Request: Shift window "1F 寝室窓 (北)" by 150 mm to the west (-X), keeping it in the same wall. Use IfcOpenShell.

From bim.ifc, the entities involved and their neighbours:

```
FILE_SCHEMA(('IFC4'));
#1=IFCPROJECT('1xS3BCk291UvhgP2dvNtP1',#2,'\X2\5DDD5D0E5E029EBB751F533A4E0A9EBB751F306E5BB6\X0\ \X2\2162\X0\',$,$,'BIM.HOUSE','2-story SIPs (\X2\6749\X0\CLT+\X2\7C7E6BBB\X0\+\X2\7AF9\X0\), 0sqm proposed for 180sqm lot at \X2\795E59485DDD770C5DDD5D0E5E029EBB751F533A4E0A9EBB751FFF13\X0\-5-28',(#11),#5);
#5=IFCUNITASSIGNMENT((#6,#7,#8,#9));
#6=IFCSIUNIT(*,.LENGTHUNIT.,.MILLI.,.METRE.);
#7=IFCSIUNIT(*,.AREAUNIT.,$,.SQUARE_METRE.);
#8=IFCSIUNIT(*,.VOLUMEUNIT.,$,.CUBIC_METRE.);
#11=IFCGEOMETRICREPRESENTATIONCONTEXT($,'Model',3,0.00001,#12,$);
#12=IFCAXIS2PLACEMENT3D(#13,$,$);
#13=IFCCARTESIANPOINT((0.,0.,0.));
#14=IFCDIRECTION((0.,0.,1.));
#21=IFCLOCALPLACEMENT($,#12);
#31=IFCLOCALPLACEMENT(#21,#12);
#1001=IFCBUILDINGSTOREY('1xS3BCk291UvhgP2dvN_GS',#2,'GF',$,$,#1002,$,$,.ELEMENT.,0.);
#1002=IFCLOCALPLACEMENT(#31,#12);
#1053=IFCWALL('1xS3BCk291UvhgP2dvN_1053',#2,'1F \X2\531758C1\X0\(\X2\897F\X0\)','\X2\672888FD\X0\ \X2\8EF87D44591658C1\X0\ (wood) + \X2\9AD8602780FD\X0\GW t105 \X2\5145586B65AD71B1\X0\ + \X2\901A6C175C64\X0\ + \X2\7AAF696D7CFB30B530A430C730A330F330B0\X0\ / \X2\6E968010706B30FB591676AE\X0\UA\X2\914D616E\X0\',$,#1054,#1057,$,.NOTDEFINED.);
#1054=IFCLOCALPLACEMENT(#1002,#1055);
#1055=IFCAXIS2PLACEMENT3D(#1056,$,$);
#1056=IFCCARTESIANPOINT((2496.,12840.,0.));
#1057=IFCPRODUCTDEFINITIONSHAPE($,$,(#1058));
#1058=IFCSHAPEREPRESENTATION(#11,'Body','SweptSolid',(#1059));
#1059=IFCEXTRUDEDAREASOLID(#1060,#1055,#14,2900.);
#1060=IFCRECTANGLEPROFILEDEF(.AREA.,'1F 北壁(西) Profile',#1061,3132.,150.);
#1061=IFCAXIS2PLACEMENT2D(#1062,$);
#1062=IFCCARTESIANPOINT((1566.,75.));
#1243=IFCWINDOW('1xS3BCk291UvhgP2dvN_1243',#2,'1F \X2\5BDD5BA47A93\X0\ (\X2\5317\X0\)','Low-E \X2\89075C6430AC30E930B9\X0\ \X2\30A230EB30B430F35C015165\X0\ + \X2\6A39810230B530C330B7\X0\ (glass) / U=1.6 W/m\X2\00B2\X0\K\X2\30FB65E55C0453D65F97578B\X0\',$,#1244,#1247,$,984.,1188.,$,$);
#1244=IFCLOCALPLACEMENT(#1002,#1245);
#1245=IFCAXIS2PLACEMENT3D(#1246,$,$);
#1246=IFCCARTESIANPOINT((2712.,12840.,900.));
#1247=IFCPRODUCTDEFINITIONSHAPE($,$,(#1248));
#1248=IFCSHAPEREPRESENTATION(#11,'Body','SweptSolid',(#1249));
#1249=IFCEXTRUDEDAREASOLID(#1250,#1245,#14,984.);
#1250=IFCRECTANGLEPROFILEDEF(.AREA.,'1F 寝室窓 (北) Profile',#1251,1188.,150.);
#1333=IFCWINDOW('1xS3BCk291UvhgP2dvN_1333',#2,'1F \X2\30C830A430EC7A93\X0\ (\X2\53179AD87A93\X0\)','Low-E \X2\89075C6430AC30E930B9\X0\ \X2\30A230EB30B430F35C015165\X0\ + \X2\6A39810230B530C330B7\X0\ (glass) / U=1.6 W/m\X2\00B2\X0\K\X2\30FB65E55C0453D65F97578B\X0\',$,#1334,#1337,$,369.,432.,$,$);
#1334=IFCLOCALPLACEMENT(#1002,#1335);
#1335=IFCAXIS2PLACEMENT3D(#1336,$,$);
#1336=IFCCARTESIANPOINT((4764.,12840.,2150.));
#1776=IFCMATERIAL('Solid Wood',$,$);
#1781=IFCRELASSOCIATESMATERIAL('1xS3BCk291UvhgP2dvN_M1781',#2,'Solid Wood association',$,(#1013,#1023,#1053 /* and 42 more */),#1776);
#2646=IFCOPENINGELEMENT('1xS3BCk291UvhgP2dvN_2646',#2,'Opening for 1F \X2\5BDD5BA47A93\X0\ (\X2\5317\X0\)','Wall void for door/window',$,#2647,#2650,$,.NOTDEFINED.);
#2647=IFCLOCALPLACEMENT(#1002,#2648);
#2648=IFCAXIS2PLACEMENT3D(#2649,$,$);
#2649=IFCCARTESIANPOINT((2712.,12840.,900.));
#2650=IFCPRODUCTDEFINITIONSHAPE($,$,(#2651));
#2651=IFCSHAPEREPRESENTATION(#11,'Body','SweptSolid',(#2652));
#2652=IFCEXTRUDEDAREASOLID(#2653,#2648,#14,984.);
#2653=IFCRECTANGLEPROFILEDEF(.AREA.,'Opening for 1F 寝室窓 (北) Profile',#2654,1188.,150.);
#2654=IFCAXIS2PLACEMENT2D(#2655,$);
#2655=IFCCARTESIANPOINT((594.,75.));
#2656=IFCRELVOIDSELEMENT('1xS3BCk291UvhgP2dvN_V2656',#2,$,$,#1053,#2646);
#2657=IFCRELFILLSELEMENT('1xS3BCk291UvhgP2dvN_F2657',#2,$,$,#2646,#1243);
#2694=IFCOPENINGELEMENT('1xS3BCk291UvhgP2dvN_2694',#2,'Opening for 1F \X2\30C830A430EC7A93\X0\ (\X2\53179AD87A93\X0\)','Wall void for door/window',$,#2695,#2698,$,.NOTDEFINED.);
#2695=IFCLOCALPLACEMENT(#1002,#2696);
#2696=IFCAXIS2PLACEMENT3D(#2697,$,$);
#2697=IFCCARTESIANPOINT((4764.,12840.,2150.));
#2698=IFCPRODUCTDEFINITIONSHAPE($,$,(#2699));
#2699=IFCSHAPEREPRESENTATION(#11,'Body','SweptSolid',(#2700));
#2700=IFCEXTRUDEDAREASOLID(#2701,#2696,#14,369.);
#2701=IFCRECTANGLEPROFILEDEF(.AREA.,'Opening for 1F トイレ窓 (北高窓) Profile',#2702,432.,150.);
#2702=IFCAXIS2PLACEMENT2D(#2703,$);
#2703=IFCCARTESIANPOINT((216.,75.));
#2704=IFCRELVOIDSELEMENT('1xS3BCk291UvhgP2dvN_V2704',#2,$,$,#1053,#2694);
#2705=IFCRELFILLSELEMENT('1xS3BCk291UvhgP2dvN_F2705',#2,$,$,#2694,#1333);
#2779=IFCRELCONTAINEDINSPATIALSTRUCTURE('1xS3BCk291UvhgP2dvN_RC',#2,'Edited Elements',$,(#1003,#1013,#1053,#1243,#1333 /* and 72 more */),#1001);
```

```python
import ifcopenshell
import ifcopenshell.api.geometry
import ifcopenshell.util.placement

model = ifcopenshell.open("bim.ifc")

window = model.by_id(1243)
opening = window.FillsVoids[0].RelatingOpeningElement
wall = opening.VoidsElements[0].RelatingBuildingElement

wall_matrix = ifcopenshell.util.placement.get_local_placement(wall.ObjectPlacement)
shift = wall_matrix[:3, 0] * -150.0
before = ifcopenshell.util.placement.get_local_placement(window.ObjectPlacement)[:3, 3].copy()

# The window is not placed relative to its opening, so move both.
for product in (opening, window):
    matrix = ifcopenshell.util.placement.get_local_placement(product.ObjectPlacement)
    matrix[:3, 3] += shift
    ifcopenshell.api.geometry.edit_object_placement(model, product=product, matrix=matrix, is_si=False)

after = ifcopenshell.util.placement.get_local_placement(window.ObjectPlacement)[:3, 3]
print("window moved by", (after - before).round(3) + 0.0)

model.write("bim_edited.ifc")
```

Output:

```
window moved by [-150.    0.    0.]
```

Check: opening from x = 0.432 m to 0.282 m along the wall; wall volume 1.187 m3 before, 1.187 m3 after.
